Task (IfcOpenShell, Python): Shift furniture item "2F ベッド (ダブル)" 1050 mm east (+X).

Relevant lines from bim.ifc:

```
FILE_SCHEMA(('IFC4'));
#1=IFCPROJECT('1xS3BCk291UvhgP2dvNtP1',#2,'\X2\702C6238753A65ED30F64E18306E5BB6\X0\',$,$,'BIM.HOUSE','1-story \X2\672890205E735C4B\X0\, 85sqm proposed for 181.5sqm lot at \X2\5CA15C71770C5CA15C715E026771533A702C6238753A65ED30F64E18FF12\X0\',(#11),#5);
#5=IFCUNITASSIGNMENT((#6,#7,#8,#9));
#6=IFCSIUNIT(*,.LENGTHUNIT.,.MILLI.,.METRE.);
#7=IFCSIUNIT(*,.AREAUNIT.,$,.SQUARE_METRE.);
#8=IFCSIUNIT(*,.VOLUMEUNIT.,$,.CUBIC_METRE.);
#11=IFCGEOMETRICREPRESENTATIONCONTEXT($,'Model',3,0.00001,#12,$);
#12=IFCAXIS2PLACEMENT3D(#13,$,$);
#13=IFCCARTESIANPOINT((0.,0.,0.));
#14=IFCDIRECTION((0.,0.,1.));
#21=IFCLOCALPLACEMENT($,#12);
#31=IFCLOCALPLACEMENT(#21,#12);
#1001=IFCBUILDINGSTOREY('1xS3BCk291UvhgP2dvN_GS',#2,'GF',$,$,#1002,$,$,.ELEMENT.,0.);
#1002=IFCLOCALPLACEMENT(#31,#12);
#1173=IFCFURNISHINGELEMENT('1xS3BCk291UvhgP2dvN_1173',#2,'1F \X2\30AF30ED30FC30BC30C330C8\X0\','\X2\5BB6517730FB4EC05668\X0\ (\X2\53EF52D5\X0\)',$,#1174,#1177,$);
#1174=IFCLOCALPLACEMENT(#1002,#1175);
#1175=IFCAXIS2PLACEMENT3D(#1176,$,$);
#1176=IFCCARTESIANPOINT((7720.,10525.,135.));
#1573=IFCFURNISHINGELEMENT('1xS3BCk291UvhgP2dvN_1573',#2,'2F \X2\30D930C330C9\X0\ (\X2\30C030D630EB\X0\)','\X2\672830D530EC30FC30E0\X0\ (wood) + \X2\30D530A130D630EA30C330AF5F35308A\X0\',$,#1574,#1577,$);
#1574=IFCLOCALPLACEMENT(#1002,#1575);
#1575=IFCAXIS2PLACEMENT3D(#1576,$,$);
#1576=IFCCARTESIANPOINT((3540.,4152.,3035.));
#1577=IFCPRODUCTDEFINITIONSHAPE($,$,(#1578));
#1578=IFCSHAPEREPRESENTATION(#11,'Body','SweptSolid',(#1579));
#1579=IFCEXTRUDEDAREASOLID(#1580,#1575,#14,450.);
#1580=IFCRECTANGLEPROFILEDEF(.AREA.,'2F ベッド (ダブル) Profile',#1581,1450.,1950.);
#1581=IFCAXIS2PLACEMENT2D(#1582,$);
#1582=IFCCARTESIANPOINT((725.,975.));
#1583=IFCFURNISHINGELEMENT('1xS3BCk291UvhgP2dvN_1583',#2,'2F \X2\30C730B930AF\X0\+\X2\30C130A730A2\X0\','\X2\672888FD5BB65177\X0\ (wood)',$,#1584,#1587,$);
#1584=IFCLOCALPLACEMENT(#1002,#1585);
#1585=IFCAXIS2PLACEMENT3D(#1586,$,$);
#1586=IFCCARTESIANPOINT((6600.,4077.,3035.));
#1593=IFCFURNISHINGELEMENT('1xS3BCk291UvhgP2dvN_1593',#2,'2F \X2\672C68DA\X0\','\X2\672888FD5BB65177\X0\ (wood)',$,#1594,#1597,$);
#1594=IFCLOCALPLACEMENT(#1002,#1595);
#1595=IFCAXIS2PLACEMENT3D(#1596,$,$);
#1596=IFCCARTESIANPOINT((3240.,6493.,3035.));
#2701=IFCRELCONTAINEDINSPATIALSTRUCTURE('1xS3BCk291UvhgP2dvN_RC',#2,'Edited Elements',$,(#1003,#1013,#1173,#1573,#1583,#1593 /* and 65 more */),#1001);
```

```python
import ifcopenshell
import ifcopenshell.api.geometry
import ifcopenshell.util.placement
import ifcopenshell.util.unit

model = ifcopenshell.open("bim.ifc")
unit_scale = ifcopenshell.util.unit.calculate_unit_scale(model)

item = model.by_id(1573)
matrix = ifcopenshell.util.placement.get_local_placement(item.ObjectPlacement)
matrix[0, 3] += 1.05 / unit_scale
ifcopenshell.api.geometry.edit_object_placement(model, product=item, matrix=matrix, is_si=False)

print(ifcopenshell.util.placement.get_local_placement(item.ObjectPlacement).round(3) + 0.0)

model.write("bim_rev.ifc")
```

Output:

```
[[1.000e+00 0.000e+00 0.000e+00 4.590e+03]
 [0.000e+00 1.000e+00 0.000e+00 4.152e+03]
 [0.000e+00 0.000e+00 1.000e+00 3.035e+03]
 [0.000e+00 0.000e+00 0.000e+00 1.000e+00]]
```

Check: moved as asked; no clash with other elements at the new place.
